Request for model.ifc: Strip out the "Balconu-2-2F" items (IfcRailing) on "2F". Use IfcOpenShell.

First a look at what the model holds.

```python
import ifcopenshell
import ifcopenshell.util.element

model = ifcopenshell.open("model.ifc")
print(model.schema)
storey = next(s for s in model.by_type("IfcBuildingStorey") if s.Name == "2F")
railings = [e for e in ifcopenshell.util.element.get_decomposition(storey) if e.is_a("IfcRailing")]
seen = {}
for e in railings:
    element_type = ifcopenshell.util.element.get_type(e)
    name = element_type.Name if element_type not in (None, e) else None
    seen[name] = seen.get(name, 0) + 1
for name, count in sorted(seen.items(), key=str):
    print(count, "x", name)
```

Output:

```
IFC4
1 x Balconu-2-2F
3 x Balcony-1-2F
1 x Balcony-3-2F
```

```python
import ifcopenshell
import ifcopenshell.api.root
import ifcopenshell.util.element

model = ifcopenshell.open("model.ifc")

storey = next(s for s in model.by_type("IfcBuildingStorey") if s.Name == "2F")
railings = [e for e in ifcopenshell.util.element.get_decomposition(storey) if e.is_a("IfcRailing")]
targets = [e for e in railings if (t := ifcopenshell.util.element.get_type(e)) not in (None, e) and t.Name == "Balconu-2-2F"]

for e in targets:
    ifcopenshell.api.root.remove_product(model, product=e)
print(len(targets), "removed")

model.write("model_rev.ifc")
```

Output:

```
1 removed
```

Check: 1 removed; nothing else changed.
